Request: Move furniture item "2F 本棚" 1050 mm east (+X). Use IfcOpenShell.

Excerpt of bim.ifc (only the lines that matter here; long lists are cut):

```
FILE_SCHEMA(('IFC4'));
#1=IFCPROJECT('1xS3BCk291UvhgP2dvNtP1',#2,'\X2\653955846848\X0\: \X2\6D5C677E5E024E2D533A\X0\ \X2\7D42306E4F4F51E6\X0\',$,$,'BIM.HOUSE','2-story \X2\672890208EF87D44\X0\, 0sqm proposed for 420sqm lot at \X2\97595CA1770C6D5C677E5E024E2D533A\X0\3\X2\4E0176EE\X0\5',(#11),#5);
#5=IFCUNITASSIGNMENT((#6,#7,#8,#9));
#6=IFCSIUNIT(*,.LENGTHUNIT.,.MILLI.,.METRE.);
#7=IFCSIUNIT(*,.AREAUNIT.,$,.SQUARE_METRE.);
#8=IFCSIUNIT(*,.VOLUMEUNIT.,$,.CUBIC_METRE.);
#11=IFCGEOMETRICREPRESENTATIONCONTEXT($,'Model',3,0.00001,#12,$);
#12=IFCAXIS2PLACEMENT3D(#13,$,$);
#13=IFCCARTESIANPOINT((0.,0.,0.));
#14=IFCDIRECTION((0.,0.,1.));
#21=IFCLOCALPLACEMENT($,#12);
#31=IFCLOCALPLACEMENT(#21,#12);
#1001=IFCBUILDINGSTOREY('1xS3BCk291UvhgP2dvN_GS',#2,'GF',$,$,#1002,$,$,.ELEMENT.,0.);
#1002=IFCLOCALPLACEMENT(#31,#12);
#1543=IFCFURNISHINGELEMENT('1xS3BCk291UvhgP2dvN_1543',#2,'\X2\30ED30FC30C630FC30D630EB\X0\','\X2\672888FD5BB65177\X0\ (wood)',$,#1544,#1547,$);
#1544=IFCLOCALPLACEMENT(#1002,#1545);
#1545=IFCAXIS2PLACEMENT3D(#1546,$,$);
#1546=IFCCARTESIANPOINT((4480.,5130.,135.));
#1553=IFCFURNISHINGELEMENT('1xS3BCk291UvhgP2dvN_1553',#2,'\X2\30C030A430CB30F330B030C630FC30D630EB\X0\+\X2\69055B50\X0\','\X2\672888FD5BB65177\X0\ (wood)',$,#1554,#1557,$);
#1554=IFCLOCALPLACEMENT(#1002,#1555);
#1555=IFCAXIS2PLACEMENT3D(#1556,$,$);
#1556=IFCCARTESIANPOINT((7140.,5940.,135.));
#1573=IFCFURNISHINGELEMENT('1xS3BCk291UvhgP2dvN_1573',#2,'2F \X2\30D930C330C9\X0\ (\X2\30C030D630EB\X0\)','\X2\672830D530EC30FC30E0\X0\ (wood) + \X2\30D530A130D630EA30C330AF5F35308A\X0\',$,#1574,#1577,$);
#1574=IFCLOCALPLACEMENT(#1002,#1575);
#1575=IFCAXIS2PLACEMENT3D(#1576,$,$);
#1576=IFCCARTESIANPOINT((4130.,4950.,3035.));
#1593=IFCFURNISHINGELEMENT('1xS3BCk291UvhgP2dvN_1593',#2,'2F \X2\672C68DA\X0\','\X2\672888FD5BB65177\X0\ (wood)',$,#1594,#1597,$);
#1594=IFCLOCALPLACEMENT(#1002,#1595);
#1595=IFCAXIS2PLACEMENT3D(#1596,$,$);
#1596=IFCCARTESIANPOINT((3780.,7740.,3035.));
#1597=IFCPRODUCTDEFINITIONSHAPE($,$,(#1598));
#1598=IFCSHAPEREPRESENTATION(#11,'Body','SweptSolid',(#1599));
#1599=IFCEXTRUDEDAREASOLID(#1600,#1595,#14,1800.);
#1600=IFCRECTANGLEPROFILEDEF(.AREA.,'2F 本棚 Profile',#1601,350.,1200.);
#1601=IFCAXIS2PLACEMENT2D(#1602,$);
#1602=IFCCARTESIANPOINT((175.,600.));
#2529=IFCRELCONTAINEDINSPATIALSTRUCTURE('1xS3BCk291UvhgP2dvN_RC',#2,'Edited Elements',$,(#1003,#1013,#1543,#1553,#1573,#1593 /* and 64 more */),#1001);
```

```python
import ifcopenshell
import ifcopenshell.api.geometry
import ifcopenshell.util.placement
import ifcopenshell.util.unit

model = ifcopenshell.open("bim.ifc")
unit_scale = ifcopenshell.util.unit.calculate_unit_scale(model)

item = model.by_guid("1xS3BCk291UvhgP2dvN_1593")
matrix = ifcopenshell.util.placement.get_local_placement(item.ObjectPlacement)
matrix[0, 3] += 1.05 / unit_scale
ifcopenshell.api.geometry.edit_object_placement(model, product=item, matrix=matrix, is_si=False)

print(ifcopenshell.util.placement.get_local_placement(item.ObjectPlacement).round(3) + 0.0)

model.write("bim-out.ifc")
```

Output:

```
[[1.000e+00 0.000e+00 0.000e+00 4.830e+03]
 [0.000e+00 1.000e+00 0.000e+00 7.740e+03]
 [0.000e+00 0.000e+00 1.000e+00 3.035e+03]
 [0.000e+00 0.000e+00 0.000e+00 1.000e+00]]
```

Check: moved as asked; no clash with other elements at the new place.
